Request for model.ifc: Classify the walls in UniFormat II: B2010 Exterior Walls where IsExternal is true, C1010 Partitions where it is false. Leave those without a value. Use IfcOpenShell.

First a look at what the model holds.

```python
import ifcopenshell
import ifcopenshell.util.element

model = ifcopenshell.open("model.ifc")
print(model.schema)
print("classifications:", [c.Name for c in model.by_type("IfcClassification")])
values = [ifcopenshell.util.element.get_pset(e, "Pset_WallCommon", "IsExternal") for e in model.by_type("IfcWall")]
for value in (True, False, None):
    print("IsExternal", value, values.count(value))
```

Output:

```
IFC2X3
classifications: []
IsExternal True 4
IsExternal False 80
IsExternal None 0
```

```python
import ifcopenshell
import ifcopenshell.api.classification
import ifcopenshell.util.element

model = ifcopenshell.open("model.ifc")

# IFC2X3 requires Source and Edition and has no link from the project to the system.
system = model.create_entity("IfcClassification", Source="ASTM", Edition="E1557", Name="UniFormat II")

walls = model.by_type("IfcWall")
external = {e: ifcopenshell.util.element.get_pset(e, "Pset_WallCommon", "IsExternal") for e in walls}
for flag, code, name in ((True, "B2010", "Exterior Walls"), (False, "C1010", "Partitions")):
    products = [e for e in walls if external[e] is flag]
    ifcopenshell.api.classification.add_reference(
        model, products=products, classification=system, identification=code, name=name
    )
    print(code, len(products))

model.write("model_v2.ifc")
```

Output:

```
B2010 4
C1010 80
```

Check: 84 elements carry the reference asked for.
